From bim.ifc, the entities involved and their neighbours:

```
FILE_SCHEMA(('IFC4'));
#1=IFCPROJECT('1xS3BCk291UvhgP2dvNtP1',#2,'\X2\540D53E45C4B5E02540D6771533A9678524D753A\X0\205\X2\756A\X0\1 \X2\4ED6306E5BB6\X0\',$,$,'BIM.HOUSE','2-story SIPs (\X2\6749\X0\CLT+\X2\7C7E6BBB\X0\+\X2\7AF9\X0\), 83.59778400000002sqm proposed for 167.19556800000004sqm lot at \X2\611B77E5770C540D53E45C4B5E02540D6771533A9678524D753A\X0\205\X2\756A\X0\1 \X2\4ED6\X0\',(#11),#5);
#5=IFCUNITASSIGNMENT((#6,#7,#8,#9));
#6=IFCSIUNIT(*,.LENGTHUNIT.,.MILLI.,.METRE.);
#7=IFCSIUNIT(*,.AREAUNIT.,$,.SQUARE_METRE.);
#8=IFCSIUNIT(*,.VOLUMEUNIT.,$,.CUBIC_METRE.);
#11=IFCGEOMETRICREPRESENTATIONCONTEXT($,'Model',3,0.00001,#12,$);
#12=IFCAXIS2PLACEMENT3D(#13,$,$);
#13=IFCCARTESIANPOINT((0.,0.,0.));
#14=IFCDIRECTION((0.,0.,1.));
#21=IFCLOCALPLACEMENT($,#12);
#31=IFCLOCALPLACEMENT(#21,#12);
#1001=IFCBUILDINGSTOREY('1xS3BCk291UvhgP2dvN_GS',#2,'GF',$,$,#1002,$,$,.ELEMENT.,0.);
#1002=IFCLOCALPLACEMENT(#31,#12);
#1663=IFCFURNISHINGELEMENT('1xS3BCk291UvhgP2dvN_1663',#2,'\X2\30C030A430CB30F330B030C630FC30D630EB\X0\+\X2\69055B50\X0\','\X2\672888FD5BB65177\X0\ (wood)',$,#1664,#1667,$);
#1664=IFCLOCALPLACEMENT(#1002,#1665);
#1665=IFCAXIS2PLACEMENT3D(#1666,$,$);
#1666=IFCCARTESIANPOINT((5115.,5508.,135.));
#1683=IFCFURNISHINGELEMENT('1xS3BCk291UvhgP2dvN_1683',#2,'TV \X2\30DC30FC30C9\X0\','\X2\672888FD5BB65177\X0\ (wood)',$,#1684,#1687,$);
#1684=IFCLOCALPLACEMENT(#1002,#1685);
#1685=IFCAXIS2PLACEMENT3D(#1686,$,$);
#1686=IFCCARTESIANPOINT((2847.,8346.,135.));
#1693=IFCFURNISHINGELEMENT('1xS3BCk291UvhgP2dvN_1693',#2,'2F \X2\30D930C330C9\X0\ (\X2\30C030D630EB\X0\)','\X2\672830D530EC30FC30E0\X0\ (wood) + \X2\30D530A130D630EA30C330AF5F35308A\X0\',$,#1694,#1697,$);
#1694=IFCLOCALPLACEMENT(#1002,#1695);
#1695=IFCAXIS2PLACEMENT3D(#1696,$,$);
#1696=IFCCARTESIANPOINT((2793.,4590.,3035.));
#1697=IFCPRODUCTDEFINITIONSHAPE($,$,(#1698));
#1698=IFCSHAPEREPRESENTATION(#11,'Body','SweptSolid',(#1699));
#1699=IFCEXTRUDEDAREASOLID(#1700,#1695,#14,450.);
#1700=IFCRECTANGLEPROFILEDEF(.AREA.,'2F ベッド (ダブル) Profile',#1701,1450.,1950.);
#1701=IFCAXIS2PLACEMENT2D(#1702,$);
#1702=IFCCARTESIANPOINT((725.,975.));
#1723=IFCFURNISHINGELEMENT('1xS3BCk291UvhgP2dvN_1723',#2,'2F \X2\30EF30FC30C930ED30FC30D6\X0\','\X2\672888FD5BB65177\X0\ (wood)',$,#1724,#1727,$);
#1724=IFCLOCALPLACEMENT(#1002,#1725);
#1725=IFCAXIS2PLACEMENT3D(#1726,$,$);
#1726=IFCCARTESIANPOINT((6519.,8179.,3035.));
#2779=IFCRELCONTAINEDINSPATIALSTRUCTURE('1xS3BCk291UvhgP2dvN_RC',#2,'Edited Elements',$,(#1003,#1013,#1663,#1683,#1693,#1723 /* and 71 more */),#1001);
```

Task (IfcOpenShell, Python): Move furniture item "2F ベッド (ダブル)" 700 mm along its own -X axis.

```python
import ifcopenshell
import ifcopenshell.api.geometry
import ifcopenshell.util.placement
import ifcopenshell.util.unit

model = ifcopenshell.open("bim.ifc")
unit_scale = ifcopenshell.util.unit.calculate_unit_scale(model)

item = model.by_id(1693)
matrix = ifcopenshell.util.placement.get_local_placement(item.ObjectPlacement)
matrix[:3, 3] -= matrix[:3, 0] * 0.7 / unit_scale
ifcopenshell.api.geometry.edit_object_placement(model, product=item, matrix=matrix, is_si=False)

print(ifcopenshell.util.placement.get_local_placement(item.ObjectPlacement).round(3) + 0.0)

model.write("bim_v2.ifc")
```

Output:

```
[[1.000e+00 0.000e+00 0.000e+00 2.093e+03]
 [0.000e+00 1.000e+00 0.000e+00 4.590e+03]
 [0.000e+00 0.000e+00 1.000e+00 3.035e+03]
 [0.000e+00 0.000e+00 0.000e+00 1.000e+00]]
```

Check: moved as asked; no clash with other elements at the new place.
